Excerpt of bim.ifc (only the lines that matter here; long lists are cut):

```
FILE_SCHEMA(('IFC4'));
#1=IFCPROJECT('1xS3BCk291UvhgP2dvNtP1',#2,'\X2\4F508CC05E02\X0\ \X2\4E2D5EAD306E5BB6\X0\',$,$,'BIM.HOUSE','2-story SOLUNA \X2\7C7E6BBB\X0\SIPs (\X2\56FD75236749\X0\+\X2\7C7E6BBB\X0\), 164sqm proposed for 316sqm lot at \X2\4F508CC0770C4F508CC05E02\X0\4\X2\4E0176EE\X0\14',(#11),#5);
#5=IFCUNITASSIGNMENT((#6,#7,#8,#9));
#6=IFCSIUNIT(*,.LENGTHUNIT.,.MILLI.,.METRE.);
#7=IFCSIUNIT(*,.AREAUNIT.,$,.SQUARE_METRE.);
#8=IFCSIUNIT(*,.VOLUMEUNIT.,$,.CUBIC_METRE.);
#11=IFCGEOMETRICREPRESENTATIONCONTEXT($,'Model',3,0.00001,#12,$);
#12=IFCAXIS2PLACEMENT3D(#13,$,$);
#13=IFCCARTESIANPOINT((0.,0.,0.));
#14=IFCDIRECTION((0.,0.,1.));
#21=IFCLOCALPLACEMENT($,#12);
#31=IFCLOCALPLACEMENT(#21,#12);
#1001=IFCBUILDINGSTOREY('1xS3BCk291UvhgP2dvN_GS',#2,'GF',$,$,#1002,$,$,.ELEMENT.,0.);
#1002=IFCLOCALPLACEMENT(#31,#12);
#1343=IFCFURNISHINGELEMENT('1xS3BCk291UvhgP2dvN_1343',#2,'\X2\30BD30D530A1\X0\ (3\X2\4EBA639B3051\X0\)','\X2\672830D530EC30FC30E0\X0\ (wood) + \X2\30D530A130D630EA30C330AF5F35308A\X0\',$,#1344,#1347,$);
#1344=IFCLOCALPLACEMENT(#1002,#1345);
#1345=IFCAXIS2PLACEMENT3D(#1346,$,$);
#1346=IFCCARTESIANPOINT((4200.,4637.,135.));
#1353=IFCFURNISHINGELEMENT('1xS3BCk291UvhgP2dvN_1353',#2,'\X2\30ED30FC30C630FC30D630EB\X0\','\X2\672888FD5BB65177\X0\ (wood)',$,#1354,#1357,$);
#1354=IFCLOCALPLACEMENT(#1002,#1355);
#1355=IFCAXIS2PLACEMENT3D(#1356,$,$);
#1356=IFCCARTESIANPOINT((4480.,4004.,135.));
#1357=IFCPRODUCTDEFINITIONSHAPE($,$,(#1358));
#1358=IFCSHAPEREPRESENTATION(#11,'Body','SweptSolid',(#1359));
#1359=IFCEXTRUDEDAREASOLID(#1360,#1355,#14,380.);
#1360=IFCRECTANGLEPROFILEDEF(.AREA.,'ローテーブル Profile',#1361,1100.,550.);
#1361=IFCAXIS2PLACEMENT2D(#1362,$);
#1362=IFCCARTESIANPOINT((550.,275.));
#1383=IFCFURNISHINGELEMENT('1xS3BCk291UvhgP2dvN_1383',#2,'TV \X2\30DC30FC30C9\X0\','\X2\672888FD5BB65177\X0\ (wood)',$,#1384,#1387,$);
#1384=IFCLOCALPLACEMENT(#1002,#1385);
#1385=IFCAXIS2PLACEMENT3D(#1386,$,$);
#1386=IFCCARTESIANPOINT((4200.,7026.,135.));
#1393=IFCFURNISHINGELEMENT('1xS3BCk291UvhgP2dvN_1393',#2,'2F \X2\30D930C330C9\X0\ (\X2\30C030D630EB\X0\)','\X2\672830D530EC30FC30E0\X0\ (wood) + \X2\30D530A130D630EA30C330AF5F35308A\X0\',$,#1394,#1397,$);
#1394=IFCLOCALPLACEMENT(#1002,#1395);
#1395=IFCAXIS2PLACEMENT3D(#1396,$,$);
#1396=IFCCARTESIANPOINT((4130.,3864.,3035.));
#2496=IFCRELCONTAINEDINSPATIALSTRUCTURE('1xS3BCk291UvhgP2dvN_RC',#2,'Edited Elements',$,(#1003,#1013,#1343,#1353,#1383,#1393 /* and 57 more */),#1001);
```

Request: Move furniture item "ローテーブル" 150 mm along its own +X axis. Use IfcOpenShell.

```python
import ifcopenshell
import ifcopenshell.api.geometry
import ifcopenshell.util.placement
import ifcopenshell.util.unit

model = ifcopenshell.open("bim.ifc")
unit_scale = ifcopenshell.util.unit.calculate_unit_scale(model)

item = model.by_guid("1xS3BCk291UvhgP2dvN_1353")
matrix = ifcopenshell.util.placement.get_local_placement(item.ObjectPlacement)
matrix[:3, 3] += matrix[:3, 0] * 0.15 / unit_scale
ifcopenshell.api.geometry.edit_object_placement(model, product=item, matrix=matrix, is_si=False)

print(ifcopenshell.util.placement.get_local_placement(item.ObjectPlacement).round(3) + 0.0)

model.write("bim-out.ifc")
```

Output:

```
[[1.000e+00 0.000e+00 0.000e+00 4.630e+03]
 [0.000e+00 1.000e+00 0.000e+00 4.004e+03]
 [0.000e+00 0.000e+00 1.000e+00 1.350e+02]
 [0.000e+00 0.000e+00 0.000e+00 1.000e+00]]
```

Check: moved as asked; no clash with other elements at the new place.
